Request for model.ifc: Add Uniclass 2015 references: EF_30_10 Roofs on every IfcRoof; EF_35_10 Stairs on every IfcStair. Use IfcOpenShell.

First a look at what the model holds.

```python
import ifcopenshell

model = ifcopenshell.open("model.ifc")
print(model.schema)
print("classifications:", [c.Name for c in model.by_type("IfcClassification")])
for ifc_class in ("IfcDoor", "IfcRoof", "IfcStair", "IfcWall", "IfcWindow"):
    print(ifc_class, len(model.by_type(ifc_class)))
```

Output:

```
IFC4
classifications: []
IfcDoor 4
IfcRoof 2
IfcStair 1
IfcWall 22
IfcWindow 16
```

```python
import ifcopenshell
import ifcopenshell.api.classification

model = ifcopenshell.open("model.ifc")

system = ifcopenshell.api.classification.add_classification(model, classification="Uniclass 2015")

codes = {
    "IfcRoof": ("EF_30_10", "Roofs"),
    "IfcStair": ("EF_35_10", "Stairs"),
}
for ifc_class, (code, name) in codes.items():
    products = model.by_type(ifc_class)
    ifcopenshell.api.classification.add_reference(
        model, products=products, classification=system, identification=code, name=name
    )
    print(code, len(products))

model.write("model_v2.ifc")
```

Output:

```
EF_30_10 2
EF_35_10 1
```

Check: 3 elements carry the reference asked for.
